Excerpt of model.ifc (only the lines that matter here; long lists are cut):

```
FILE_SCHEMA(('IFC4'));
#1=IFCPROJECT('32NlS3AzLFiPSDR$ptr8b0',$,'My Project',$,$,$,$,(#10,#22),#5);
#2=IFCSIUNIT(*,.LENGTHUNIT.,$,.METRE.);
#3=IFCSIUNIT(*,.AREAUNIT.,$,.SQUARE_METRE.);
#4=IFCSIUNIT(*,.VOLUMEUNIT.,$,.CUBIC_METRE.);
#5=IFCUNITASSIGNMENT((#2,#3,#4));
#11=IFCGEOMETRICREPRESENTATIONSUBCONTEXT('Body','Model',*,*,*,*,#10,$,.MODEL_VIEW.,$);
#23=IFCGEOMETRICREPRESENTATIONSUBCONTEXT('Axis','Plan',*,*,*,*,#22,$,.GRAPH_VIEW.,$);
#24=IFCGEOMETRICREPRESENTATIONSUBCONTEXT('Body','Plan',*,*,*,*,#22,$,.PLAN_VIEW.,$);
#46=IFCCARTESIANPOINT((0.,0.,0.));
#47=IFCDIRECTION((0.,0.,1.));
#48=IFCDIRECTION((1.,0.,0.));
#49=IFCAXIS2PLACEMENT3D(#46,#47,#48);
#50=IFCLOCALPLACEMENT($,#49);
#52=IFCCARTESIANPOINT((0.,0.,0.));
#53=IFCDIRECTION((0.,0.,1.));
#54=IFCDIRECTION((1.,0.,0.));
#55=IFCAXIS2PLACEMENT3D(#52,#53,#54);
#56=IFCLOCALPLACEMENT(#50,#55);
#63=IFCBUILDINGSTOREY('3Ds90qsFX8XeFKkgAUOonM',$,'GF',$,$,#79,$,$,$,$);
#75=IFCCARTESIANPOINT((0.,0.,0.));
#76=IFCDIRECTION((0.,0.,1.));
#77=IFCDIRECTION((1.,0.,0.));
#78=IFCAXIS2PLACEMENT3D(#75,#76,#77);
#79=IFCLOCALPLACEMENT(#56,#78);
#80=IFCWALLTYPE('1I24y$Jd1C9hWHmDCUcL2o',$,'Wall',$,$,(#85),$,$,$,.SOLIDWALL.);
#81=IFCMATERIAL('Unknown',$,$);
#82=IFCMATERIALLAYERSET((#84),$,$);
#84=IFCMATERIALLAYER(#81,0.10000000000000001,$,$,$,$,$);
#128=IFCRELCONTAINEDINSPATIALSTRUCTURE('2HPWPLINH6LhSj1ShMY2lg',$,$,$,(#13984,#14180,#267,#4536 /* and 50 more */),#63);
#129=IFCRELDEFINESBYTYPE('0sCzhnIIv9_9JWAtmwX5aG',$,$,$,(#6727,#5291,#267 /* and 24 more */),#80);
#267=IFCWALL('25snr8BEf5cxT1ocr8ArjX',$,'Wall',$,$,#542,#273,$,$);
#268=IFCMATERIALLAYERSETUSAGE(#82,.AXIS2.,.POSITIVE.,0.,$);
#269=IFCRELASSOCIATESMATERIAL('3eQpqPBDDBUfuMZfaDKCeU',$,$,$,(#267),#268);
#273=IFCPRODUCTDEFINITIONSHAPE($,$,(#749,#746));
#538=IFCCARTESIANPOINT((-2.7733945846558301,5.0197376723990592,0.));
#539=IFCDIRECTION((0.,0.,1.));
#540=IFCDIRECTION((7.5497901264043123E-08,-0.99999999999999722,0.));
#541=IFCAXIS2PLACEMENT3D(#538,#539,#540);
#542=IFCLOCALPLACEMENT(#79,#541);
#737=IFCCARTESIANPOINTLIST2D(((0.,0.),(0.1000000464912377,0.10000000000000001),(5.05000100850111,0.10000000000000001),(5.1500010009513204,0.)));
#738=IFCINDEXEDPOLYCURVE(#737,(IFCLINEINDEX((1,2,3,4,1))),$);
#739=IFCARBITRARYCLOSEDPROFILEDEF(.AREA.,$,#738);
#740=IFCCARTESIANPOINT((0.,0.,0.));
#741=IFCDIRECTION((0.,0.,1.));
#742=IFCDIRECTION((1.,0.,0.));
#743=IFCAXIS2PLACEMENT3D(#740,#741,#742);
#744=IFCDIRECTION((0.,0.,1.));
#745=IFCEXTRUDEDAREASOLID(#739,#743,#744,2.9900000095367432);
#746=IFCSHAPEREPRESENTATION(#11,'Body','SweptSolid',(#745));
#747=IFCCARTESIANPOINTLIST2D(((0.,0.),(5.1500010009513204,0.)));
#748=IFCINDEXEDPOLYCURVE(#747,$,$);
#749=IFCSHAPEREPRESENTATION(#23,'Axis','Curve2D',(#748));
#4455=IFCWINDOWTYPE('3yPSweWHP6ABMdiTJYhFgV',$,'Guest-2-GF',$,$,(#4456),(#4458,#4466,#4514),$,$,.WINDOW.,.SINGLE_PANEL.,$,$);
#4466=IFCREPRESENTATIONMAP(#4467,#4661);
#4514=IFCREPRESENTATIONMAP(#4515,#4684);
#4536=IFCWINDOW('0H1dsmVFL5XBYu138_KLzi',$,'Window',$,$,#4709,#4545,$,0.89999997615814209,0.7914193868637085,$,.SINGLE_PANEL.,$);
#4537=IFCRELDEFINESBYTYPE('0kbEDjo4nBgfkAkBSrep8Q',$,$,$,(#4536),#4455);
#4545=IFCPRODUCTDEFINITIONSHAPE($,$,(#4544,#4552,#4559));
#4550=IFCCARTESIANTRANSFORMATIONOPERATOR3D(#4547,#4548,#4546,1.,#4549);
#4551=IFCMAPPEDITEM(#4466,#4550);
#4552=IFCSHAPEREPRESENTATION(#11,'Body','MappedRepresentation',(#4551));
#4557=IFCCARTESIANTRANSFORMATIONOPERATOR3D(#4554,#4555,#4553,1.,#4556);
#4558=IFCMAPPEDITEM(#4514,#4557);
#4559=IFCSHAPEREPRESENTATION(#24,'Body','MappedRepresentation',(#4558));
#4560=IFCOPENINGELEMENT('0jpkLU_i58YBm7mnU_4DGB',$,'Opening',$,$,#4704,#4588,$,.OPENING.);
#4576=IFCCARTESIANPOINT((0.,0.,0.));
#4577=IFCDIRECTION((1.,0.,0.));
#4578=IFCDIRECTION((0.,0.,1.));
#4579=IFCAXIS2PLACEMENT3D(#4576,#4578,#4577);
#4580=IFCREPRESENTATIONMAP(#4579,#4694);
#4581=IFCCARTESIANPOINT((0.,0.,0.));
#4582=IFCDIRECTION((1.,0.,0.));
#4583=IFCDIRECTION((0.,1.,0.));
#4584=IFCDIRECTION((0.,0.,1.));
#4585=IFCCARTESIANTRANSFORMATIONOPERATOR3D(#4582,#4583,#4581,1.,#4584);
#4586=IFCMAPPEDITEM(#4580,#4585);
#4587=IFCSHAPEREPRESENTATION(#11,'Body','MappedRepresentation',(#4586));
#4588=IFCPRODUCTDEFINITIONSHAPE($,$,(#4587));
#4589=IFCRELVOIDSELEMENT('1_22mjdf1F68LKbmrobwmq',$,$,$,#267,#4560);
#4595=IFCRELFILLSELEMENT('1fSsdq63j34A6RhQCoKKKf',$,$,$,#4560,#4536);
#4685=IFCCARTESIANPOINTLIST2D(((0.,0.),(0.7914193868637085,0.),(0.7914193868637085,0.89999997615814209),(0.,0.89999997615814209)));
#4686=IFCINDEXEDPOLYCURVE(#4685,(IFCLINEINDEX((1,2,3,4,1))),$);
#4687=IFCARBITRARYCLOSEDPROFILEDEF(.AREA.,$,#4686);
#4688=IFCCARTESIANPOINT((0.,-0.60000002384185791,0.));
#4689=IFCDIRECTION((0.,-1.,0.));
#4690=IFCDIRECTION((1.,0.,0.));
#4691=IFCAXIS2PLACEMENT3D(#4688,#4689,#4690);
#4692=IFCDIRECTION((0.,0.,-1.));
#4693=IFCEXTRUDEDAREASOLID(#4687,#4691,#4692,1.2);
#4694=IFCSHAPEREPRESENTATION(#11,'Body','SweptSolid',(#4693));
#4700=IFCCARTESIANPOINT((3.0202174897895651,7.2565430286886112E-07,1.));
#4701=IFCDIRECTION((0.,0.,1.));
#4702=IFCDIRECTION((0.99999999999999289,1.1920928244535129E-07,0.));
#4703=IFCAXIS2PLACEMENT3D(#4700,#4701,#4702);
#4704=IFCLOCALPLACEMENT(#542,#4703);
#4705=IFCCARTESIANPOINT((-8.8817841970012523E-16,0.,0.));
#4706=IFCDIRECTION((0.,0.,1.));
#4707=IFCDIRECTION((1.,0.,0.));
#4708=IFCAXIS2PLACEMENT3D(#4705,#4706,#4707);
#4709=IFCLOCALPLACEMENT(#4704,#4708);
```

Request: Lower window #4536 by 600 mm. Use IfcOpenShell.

```python
import numpy as np
import ifcopenshell
import ifcopenshell.api.geometry
import ifcopenshell.util.placement
import ifcopenshell.util.unit

model = ifcopenshell.open("model.ifc")
unit_scale = ifcopenshell.util.unit.calculate_unit_scale(model)

window = model.by_guid("0H1dsmVFL5XBYu138_KLzi")
opening = window.FillsVoids[0].RelatingOpeningElement
dz = -0.6 / unit_scale

shift = np.array([0.0, 0.0, dz])
# The window is placed relative to its opening, so it follows when the opening moves.
matrix = ifcopenshell.util.placement.get_local_placement(opening.ObjectPlacement)
matrix[:3, 3] += shift
ifcopenshell.api.geometry.edit_object_placement(
    model, product=opening, matrix=matrix, is_si=False, should_transform_children=True
)

print(f"moved by {dz * unit_scale:+.3f} m")

model.write("model_v2.ifc")
```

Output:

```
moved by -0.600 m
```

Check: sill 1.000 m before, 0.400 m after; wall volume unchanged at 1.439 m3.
